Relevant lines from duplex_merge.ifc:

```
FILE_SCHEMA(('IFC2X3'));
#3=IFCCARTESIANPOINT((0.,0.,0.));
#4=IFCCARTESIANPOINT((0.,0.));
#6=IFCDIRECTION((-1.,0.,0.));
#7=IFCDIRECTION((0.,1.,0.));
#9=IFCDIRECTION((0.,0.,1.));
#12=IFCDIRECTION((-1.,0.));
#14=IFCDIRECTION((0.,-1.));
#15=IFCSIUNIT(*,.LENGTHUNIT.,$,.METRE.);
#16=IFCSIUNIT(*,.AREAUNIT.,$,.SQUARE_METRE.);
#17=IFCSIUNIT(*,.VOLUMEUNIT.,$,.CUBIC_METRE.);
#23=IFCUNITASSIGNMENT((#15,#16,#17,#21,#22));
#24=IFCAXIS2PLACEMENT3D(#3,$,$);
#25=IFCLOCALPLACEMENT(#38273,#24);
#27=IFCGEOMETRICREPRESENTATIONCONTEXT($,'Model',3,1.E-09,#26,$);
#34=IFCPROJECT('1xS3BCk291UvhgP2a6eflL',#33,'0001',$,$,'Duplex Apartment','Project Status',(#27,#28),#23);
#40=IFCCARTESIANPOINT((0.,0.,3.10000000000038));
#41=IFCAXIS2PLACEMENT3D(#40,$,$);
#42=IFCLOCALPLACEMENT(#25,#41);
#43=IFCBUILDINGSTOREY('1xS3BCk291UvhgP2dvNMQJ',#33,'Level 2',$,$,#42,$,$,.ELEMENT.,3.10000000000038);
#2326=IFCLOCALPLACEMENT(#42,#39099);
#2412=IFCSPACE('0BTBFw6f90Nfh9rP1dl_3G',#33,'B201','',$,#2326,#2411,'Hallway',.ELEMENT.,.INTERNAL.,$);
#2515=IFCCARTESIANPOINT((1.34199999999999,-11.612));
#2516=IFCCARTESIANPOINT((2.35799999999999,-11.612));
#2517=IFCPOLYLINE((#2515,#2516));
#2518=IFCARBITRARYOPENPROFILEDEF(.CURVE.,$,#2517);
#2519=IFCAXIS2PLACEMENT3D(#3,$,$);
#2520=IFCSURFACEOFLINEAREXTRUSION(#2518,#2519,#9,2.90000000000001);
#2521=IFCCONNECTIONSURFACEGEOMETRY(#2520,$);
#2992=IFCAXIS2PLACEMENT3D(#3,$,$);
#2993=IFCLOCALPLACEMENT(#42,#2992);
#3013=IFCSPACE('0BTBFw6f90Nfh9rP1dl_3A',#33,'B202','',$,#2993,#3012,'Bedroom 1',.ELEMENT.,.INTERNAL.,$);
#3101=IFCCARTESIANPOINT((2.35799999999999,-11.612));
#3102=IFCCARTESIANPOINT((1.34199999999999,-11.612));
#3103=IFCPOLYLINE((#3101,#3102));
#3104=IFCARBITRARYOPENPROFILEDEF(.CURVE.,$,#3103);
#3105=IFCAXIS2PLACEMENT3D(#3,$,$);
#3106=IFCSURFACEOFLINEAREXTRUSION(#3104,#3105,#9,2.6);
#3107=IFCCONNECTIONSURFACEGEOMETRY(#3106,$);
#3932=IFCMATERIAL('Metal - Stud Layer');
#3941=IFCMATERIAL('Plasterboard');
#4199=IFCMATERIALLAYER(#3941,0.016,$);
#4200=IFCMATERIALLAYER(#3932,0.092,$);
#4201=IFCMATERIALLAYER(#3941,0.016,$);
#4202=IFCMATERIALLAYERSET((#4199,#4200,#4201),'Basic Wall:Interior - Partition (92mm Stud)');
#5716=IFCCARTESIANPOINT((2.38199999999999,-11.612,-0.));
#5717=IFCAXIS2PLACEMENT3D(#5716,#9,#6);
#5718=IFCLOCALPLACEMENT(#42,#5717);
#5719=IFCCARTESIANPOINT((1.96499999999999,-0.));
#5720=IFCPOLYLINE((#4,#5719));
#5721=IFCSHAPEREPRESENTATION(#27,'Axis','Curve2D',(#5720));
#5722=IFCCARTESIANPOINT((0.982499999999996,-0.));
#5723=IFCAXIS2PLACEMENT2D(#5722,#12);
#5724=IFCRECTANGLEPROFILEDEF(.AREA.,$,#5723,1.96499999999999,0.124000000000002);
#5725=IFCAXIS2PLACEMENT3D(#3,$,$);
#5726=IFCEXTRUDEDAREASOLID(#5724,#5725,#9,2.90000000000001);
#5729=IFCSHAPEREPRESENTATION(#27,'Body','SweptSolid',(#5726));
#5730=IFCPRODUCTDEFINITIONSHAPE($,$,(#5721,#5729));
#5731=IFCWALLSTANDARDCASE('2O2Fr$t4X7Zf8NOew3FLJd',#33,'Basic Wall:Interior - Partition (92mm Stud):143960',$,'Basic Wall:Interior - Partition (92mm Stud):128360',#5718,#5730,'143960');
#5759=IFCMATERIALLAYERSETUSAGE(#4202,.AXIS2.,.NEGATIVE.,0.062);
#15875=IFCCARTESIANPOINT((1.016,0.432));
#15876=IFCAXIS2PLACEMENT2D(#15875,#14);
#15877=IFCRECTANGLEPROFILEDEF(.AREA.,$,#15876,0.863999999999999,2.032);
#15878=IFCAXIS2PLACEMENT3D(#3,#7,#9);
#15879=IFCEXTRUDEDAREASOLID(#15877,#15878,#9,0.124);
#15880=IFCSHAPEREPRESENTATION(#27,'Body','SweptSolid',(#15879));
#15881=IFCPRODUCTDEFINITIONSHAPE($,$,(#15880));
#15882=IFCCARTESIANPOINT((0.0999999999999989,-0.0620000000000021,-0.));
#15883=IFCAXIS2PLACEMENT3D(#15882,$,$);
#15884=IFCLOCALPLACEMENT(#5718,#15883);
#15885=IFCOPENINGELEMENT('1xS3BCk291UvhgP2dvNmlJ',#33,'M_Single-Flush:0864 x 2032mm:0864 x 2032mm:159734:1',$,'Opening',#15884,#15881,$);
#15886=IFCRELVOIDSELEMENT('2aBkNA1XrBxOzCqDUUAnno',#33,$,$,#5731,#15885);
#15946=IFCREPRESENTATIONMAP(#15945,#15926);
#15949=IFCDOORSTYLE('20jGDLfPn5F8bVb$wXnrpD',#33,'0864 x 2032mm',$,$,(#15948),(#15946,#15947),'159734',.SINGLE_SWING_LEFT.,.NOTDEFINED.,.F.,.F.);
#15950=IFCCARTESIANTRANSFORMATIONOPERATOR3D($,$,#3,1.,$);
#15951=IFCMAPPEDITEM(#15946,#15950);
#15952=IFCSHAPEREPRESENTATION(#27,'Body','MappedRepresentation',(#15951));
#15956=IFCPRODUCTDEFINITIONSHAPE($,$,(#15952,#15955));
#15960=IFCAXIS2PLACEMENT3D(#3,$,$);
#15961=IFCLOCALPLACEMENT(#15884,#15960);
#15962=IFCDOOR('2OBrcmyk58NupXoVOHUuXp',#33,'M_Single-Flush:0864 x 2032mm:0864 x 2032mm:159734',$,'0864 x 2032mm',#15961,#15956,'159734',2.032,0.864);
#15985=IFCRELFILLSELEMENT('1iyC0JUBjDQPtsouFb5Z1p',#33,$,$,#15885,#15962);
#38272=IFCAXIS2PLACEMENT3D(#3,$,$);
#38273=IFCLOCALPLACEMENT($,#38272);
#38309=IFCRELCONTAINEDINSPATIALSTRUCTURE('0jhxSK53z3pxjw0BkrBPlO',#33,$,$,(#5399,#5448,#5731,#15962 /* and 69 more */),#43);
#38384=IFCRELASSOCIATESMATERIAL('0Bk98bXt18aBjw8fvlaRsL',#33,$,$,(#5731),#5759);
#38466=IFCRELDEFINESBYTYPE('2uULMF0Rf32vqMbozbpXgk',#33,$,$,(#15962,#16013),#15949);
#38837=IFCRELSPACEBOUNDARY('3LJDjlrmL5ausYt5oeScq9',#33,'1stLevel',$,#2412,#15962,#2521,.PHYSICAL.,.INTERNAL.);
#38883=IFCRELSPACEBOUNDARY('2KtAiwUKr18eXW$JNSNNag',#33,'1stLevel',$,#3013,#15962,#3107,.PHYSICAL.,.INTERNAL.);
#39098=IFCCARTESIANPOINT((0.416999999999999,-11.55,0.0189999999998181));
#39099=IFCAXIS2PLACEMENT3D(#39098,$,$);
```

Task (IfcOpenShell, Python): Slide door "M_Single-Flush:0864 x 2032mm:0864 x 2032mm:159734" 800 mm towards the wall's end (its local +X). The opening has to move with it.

```python
import numpy as np
import ifcopenshell
import ifcopenshell.api.geometry
import ifcopenshell.util.placement
import ifcopenshell.util.unit

model = ifcopenshell.open("duplex_merge.ifc")
unit_scale = ifcopenshell.util.unit.calculate_unit_scale(model)

door = model.by_id(15962)
opening = door.FillsVoids[0].RelatingOpeningElement
wall = opening.VoidsElements[0].RelatingBuildingElement

wall_matrix = ifcopenshell.util.placement.get_local_placement(wall.ObjectPlacement)
shift = wall_matrix[:3, 0] * 0.8 / unit_scale
before = ifcopenshell.util.placement.get_local_placement(door.ObjectPlacement)[:3, 3].copy()

# The door is placed relative to its opening, so it follows when the opening moves.
matrix = ifcopenshell.util.placement.get_local_placement(opening.ObjectPlacement)
matrix[:3, 3] += shift
ifcopenshell.api.geometry.edit_object_placement(
    model, product=opening, matrix=matrix, is_si=False, should_transform_children=True
)

# Space boundary surfaces are stored in each space's coordinates; move them too.
for rel in door.ProvidesBoundaries:
    if not rel.ConnectionGeometry:
        continue
    surface = rel.ConnectionGeometry.SurfaceOnRelatingElement
    space_matrix = ifcopenshell.util.placement.get_local_placement(rel.RelatingSpace.ObjectPlacement)
    point = np.array(surface.Position.Location.Coordinates) + space_matrix[:3, :3].T @ shift
    surface.Position = model.createIfcAxis2Placement3D(
        model.createIfcCartesianPoint(point.tolist()), surface.Position.Axis, surface.Position.RefDirection
    )

after = ifcopenshell.util.placement.get_local_placement(door.ObjectPlacement)[:3, 3]
print("door moved by", (after - before).round(3) + 0.0)

model.write("duplex_merge_updated.ifc")
```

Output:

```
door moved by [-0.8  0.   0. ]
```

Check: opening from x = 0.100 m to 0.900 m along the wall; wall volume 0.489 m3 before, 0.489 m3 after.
